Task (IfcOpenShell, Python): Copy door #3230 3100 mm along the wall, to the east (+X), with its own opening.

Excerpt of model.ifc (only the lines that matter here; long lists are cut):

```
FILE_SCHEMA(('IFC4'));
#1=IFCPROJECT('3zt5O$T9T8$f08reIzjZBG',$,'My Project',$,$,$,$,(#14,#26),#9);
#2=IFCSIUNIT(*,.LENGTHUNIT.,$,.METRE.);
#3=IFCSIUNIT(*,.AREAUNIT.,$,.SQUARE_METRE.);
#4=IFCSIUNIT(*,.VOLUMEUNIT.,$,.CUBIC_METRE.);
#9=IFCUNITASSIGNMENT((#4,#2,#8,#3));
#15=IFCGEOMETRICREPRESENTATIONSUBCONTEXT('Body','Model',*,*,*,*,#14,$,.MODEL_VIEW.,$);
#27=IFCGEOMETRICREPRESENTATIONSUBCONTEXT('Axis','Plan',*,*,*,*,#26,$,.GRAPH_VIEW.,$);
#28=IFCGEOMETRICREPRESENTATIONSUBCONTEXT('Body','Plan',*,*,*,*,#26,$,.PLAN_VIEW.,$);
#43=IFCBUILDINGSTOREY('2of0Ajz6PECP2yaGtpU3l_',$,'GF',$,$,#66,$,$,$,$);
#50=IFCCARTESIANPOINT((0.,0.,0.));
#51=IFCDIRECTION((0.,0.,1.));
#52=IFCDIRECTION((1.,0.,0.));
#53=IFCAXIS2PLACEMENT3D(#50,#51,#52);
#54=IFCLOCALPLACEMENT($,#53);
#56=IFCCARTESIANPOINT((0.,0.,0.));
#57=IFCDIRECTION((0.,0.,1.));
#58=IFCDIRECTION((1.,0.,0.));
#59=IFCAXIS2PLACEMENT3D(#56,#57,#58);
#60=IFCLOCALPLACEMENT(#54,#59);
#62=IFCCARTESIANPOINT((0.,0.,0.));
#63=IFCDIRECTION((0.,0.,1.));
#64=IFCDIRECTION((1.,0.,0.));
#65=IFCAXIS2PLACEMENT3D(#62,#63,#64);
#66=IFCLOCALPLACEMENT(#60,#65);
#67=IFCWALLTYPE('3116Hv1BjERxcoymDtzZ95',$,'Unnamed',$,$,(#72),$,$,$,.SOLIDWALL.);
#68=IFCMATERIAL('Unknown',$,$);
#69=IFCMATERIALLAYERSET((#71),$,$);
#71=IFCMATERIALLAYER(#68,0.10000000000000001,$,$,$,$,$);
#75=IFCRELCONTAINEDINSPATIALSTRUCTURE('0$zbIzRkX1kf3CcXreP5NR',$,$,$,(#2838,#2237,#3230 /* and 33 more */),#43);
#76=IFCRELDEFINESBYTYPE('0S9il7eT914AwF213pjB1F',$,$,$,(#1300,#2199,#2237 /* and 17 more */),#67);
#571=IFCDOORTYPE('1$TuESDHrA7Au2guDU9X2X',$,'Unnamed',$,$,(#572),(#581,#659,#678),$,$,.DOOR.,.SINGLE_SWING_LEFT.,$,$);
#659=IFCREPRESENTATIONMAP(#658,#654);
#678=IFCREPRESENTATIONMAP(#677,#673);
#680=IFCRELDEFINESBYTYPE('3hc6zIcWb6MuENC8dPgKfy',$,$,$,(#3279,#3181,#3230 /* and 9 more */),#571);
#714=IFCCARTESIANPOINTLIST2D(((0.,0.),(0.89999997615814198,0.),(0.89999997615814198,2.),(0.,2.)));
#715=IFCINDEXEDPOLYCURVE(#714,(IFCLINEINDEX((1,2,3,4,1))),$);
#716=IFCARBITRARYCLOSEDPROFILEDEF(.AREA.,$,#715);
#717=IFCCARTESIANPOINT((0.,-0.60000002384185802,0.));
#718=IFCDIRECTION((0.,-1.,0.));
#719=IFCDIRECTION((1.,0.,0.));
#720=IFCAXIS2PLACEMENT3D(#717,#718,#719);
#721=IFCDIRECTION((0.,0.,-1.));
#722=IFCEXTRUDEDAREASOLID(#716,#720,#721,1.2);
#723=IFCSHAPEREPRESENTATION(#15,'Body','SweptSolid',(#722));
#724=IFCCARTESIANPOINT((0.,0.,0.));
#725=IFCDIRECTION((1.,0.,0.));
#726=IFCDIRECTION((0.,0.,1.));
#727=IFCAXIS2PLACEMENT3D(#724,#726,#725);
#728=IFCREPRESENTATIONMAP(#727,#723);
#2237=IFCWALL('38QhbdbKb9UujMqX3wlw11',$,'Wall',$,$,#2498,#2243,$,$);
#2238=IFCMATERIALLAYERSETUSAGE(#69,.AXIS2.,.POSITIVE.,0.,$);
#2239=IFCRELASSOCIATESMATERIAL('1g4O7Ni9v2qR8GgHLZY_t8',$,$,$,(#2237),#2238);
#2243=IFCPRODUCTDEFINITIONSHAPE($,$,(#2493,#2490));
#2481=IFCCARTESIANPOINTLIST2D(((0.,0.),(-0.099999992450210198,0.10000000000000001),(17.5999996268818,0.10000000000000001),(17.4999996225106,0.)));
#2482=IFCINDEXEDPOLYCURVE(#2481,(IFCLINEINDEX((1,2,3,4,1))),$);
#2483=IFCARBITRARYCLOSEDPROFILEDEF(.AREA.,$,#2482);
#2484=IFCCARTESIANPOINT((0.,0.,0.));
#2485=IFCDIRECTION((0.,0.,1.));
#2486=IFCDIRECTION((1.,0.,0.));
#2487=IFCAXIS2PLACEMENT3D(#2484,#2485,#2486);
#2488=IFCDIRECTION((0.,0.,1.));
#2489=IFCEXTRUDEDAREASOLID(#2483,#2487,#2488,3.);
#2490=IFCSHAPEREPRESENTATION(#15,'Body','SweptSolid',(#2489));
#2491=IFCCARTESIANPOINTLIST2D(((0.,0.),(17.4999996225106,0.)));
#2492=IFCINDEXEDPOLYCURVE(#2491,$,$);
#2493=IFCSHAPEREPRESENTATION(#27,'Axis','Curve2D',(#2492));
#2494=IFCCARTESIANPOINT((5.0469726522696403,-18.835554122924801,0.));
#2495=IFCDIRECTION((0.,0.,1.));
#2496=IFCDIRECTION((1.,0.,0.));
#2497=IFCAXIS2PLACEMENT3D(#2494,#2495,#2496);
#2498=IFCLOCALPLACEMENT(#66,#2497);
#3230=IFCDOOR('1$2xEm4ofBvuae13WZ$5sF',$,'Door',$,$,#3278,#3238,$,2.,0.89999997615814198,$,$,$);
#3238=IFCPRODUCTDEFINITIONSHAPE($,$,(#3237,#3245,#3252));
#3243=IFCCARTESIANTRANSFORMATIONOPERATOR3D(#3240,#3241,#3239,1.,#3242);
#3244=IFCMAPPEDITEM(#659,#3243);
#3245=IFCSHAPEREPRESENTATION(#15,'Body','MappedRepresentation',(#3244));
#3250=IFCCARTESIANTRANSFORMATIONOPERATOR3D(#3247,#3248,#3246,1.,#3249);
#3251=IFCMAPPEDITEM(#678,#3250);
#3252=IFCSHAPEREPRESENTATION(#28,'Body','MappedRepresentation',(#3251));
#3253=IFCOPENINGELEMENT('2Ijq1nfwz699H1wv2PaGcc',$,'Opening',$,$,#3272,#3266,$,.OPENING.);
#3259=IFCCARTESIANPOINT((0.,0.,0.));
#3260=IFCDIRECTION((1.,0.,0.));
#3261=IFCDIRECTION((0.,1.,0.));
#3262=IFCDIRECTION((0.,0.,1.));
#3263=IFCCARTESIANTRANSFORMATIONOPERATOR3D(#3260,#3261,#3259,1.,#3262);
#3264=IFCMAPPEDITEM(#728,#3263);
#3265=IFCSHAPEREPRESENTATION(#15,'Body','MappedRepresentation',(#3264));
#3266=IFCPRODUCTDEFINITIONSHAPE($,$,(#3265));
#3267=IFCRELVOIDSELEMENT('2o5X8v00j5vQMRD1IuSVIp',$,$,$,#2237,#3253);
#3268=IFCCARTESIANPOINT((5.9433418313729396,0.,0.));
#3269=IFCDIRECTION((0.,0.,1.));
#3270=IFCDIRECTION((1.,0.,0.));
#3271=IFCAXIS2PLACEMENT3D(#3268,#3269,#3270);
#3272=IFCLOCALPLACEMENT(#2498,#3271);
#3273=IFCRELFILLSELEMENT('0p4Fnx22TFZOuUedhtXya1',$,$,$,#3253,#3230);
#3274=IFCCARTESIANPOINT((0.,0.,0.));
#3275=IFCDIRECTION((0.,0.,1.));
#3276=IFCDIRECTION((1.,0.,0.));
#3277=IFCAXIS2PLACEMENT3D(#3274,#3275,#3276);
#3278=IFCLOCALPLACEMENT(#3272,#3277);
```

```python
import ifcopenshell
import ifcopenshell.api.feature
import ifcopenshell.api.geometry
import ifcopenshell.api.root
import ifcopenshell.geom
import ifcopenshell.util.element
import ifcopenshell.util.placement
import ifcopenshell.util.shape
import ifcopenshell.util.unit

model = ifcopenshell.open("model.ifc")
unit_scale = ifcopenshell.util.unit.calculate_unit_scale(model)
settings = ifcopenshell.geom.settings()


def volume(element):
    """Net volume in cubic metres, openings subtracted."""
    shape = ifcopenshell.geom.create_shape(settings, element)
    return ifcopenshell.util.shape.get_volume(shape.geometry)


door = model.by_guid("1$2xEm4ofBvuae13WZ$5sF")
opening = door.FillsVoids[0].RelatingOpeningElement
wall = opening.VoidsElements[0].RelatingBuildingElement
before = volume(wall)
shift = ifcopenshell.util.placement.get_local_placement(wall.ObjectPlacement)[:3, 0] * 3.1 / unit_scale

# copy_class copies the void relationship, type, container and properties, but no geometry.
new_opening = ifcopenshell.api.root.copy_class(model, product=opening)
new_opening.Representation = ifcopenshell.util.element.copy_deep(
    model, opening.Representation, exclude=["IfcGeometricRepresentationContext", "IfcRepresentationMap"]
)
new_door = ifcopenshell.api.root.copy_class(model, product=door)
new_door.Representation = ifcopenshell.util.element.copy_deep(
    model, door.Representation, exclude=["IfcGeometricRepresentationContext", "IfcRepresentationMap"]
)
ifcopenshell.api.feature.add_filling(model, opening=new_opening, element=new_door)

for old, new in ((opening, new_opening), (door, new_door)):
    matrix = ifcopenshell.util.placement.get_local_placement(old.ObjectPlacement)
    matrix[:3, 3] += shift
    ifcopenshell.api.geometry.edit_object_placement(model, product=new, matrix=matrix, is_si=False)

after = volume(wall)

print(f"wall volume {before:.3f} -> {after:.3f} m3")

model.write("model_updated.ifc")
```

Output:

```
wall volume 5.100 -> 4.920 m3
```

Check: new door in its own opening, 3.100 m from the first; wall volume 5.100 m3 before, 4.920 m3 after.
